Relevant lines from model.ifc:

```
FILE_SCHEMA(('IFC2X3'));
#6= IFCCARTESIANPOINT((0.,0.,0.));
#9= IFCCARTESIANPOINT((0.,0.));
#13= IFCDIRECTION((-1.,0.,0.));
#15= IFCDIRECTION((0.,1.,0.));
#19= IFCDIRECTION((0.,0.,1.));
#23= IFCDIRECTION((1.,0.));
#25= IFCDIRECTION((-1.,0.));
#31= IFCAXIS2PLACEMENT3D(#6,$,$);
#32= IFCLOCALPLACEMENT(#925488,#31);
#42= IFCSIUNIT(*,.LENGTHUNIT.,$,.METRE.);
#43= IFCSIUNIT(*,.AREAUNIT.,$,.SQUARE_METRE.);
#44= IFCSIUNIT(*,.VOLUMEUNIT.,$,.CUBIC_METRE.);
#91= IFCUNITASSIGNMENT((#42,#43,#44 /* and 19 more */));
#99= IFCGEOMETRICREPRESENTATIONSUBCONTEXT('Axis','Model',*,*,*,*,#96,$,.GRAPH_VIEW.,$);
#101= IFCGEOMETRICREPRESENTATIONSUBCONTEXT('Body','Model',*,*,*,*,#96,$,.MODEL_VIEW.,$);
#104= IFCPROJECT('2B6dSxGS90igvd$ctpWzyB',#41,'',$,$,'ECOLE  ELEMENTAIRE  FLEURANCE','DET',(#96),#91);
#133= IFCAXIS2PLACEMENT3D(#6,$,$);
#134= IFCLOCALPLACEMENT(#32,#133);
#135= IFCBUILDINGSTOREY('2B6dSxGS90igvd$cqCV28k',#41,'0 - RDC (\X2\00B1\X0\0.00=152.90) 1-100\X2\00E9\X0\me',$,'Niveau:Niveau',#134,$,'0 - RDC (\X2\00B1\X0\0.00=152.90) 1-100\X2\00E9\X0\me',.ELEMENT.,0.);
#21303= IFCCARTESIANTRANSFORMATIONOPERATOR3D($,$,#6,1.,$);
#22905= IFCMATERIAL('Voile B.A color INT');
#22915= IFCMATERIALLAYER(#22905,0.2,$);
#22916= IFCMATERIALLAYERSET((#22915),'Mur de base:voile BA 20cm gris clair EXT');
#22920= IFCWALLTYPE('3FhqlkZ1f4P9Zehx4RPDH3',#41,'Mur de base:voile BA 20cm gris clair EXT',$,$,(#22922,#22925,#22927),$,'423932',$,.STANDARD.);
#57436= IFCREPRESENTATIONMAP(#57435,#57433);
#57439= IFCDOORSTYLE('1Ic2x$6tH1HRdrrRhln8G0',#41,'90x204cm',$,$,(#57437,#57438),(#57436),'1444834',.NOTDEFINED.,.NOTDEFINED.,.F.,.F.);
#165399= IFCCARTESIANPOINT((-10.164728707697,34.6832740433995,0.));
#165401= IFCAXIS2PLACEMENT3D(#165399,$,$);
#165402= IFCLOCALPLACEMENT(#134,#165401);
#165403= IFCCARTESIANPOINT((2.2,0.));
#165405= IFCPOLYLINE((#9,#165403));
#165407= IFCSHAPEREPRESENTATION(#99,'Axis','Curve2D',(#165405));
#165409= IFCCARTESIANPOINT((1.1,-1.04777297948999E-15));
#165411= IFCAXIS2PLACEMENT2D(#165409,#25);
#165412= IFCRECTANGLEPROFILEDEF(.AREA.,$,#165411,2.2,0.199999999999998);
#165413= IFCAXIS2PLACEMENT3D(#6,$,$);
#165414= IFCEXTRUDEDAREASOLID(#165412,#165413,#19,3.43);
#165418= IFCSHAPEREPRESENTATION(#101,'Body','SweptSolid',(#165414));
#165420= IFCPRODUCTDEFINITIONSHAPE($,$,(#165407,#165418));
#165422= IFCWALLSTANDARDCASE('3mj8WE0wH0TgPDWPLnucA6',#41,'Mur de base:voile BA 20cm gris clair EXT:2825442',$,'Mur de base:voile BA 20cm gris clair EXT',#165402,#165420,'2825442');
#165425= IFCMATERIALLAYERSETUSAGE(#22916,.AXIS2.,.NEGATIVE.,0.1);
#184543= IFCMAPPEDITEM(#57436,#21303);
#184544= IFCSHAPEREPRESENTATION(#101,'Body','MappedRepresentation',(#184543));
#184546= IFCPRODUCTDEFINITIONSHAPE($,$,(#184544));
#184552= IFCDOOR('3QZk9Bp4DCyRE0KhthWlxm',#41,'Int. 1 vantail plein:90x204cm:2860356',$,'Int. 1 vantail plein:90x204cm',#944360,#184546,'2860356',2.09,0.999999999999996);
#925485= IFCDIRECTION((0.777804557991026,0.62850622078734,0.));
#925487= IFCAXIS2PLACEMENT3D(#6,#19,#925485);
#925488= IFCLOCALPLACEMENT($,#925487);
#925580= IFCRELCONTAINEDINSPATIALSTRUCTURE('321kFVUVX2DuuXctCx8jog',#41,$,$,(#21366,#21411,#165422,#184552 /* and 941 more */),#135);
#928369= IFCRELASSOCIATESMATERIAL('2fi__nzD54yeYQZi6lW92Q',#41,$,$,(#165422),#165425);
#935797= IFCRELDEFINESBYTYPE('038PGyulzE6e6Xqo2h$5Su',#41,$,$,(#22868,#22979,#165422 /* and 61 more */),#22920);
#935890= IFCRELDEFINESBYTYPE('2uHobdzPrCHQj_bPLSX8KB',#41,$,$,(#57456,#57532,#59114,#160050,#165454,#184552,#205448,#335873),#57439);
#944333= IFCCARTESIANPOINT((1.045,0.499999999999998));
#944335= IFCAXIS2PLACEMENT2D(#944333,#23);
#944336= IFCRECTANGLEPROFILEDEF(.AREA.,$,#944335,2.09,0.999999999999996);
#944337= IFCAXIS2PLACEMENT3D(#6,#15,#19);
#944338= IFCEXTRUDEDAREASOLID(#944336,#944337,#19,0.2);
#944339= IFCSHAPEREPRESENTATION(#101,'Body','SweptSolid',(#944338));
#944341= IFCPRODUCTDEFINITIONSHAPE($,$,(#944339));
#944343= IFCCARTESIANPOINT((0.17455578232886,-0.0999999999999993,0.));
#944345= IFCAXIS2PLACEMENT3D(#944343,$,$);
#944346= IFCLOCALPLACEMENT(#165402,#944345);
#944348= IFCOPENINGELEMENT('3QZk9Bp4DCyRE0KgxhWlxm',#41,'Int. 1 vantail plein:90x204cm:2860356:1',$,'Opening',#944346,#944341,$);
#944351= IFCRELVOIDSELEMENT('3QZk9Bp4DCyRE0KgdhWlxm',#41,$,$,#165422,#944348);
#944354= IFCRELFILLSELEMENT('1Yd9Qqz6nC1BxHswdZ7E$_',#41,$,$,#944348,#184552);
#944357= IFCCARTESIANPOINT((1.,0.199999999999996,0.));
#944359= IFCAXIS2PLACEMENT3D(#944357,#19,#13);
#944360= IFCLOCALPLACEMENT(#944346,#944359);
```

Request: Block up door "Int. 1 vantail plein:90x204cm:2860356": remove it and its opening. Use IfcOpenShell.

```python
import ifcopenshell
import ifcopenshell.api.feature
import ifcopenshell.api.root
import ifcopenshell.geom
import ifcopenshell.util.shape

model = ifcopenshell.open("model.ifc")
settings = ifcopenshell.geom.settings()


def volume(element):
    """Net volume in cubic metres, openings subtracted."""
    shape = ifcopenshell.geom.create_shape(settings, element)
    return ifcopenshell.util.shape.get_volume(shape.geometry)


door = model.by_guid("3QZk9Bp4DCyRE0KhthWlxm")
opening = door.FillsVoids[0].RelatingOpeningElement
wall = opening.VoidsElements[0].RelatingBuildingElement
before = volume(wall)

ifcopenshell.api.root.remove_product(model, product=door)
ifcopenshell.api.feature.remove_feature(model, feature=opening)

after = volume(wall)

print(f"wall volume {before:.3f} -> {after:.3f} m3")

model.write("model_updated.ifc")
```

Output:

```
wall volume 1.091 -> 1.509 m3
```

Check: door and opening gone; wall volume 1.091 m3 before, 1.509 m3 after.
